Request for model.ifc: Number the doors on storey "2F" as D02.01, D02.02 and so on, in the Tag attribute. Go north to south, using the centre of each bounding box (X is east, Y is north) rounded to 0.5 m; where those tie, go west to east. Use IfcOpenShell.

First a look at what the model holds.

```python
import ifcopenshell
import ifcopenshell.util.element
import ifcopenshell.util.placement

model = ifcopenshell.open("model.ifc")
print(model.schema)
storey = next(s for s in model.by_type("IfcBuildingStorey") if s.Name == "2F")
doors = [e for e in ifcopenshell.util.element.get_decomposition(storey) if e.is_a("IfcDoor")]
for e in sorted(doors, key=lambda e: e.id()):
    origin = ifcopenshell.util.placement.get_local_placement(e.ObjectPlacement)[:3, 3]
    print(e.id(), e.Tag, e.Name, origin.round(2) + 0.0, sep=" | ")
```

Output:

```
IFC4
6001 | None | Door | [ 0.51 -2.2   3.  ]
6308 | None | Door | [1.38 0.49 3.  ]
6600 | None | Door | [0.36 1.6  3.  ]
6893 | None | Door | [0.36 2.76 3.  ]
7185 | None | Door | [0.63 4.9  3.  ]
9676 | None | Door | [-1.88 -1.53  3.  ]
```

```python
import ifcopenshell
import ifcopenshell.geom
import ifcopenshell.util.element
import ifcopenshell.util.shape

model = ifcopenshell.open("model.ifc")
settings = ifcopenshell.geom.settings()
settings.set("use-world-coords", True)


def centre(element):
    shape = ifcopenshell.geom.create_shape(settings, element)
    return ifcopenshell.util.shape.get_bbox_centroid(shape.geometry)


storey = next(s for s in model.by_type("IfcBuildingStorey") if s.Name == "2F")
doors = [e for e in ifcopenshell.util.element.get_decomposition(storey) if e.is_a("IfcDoor")]

# Insertion points can sit at a corner or the storey origin, so sort by the geometry (in metres).
centres = {e: centre(e) for e in doors}
doors.sort(key=lambda e: (-round(centres[e][1] / 0.5), centres[e][0]))

for i, e in enumerate(doors, start=1):
    number = f"D02.{i:02d}"
    e.Tag = number
    print(e.id(), number)

model.write("model_v2.ifc")
```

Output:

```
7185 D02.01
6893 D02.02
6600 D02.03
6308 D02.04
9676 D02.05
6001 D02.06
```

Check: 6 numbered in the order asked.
